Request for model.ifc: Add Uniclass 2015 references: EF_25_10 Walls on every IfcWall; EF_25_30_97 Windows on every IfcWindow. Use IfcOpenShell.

First a look at what the model holds.

```python
import ifcopenshell

model = ifcopenshell.open("model.ifc")
print(model.schema)
print("classifications:", [c.Name for c in model.by_type("IfcClassification")])
for ifc_class in ("IfcDoor", "IfcRoof", "IfcStair", "IfcWall", "IfcWindow"):
    print(ifc_class, len(model.by_type(ifc_class)))
```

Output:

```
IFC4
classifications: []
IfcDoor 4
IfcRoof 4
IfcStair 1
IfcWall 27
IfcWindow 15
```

```python
import ifcopenshell
import ifcopenshell.api.classification

model = ifcopenshell.open("model.ifc")

system = ifcopenshell.api.classification.add_classification(model, classification="Uniclass 2015")

codes = {
    "IfcWall": ("EF_25_10", "Walls"),
    "IfcWindow": ("EF_25_30_97", "Windows"),
}
for ifc_class, (code, name) in codes.items():
    products = model.by_type(ifc_class)
    ifcopenshell.api.classification.add_reference(
        model, products=products, classification=system, identification=code, name=name
    )
    print(code, len(products))

model.write("model_rev.ifc")
```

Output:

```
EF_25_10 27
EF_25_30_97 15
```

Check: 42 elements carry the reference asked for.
